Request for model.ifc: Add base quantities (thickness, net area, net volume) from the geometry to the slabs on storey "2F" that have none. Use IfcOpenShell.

First a look at what the model holds.

```python
import ifcopenshell
import ifcopenshell.util.element
import ifcopenshell.util.unit

model = ifcopenshell.open("model.ifc")
print(model.schema)
for unit_type in ("LENGTHUNIT", "AREAUNIT", "VOLUMEUNIT"):
    print(unit_type, ifcopenshell.util.unit.calculate_unit_scale(model, unit_type))
storey = next(s for s in model.by_type("IfcBuildingStorey") if s.Name == "2F")
slabs = [e for e in ifcopenshell.util.element.get_decomposition(storey) if e.is_a("IfcSlab")]
for e in sorted(slabs, key=lambda e: e.id()):
    print(e.id(), e.is_a(), e.Name, list(ifcopenshell.util.element.get_psets(e, qtos_only=True)), sep=" | ")
```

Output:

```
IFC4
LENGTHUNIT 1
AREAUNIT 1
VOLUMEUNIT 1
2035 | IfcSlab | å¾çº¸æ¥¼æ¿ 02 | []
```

```python
import ifcopenshell
import ifcopenshell.api.pset
import ifcopenshell.geom
import ifcopenshell.util.element
import ifcopenshell.util.shape
import ifcopenshell.util.unit

model = ifcopenshell.open("model.ifc")
unit_scale = ifcopenshell.util.unit.calculate_unit_scale(model)
area_scale = ifcopenshell.util.unit.calculate_unit_scale(model, "AREAUNIT")
volume_scale = ifcopenshell.util.unit.calculate_unit_scale(model, "VOLUMEUNIT")
settings = ifcopenshell.geom.settings()

storey = next(s for s in model.by_type("IfcBuildingStorey") if s.Name == "2F")
slabs = [e for e in ifcopenshell.util.element.get_decomposition(storey) if e.is_a("IfcSlab")]

for e in sorted(slabs, key=lambda e: e.id()):
    if ifcopenshell.util.element.get_psets(e, qtos_only=True, should_inherit=False):
        continue
    # Geometry comes back in metres, in the element's own axes.
    shape = ifcopenshell.geom.create_shape(settings, e)
    values = {
        "Width": ifcopenshell.util.shape.get_z(shape.geometry) / unit_scale,
        "NetArea": ifcopenshell.util.shape.get_footprint_area(shape.geometry) / area_scale,
        "NetVolume": ifcopenshell.util.shape.get_volume(shape.geometry) / volume_scale,
    }
    qto = ifcopenshell.api.pset.add_qto(model, product=e, name="Qto_SlabBaseQuantities")
    ifcopenshell.api.pset.edit_qto(model, qto=qto, properties=values)
    print(e.id(), {k: round(v, 3) for k, v in values.items()})

model.write("model_updated.ifc")
```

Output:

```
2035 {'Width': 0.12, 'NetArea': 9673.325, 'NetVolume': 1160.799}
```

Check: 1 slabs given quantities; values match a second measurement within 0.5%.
